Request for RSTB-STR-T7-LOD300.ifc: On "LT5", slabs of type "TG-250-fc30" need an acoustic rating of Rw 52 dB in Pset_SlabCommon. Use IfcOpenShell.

First a look at what the model holds.

```python
import ifcopenshell
import ifcopenshell.util.element

model = ifcopenshell.open("RSTB-STR-T7-LOD300.ifc")
print(model.schema)
storey = next(s for s in model.by_type("IfcBuildingStorey") if s.Name == "LT5")
slabs = [e for e in ifcopenshell.util.element.get_decomposition(storey) if e.is_a("IfcSlab")]
seen = {}
for e in slabs:
    element_type = ifcopenshell.util.element.get_type(e)
    key = (element_type.Name if element_type != e and element_type else None, ifcopenshell.util.element.get_pset(e, "Pset_SlabCommon", "AcousticRating"))
    seen[key] = seen.get(key, 0) + 1
for (name, value), count in sorted(seen.items(), key=str):
    print(count, "x", name, "|", value)
```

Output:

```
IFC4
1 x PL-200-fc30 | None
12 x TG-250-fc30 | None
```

```python
import ifcopenshell
import ifcopenshell.api.pset
import ifcopenshell.util.element

model = ifcopenshell.open("RSTB-STR-T7-LOD300.ifc")

storey = next(s for s in model.by_type("IfcBuildingStorey") if s.Name == "LT5")
slabs = [e for e in ifcopenshell.util.element.get_decomposition(storey) if e.is_a("IfcSlab")]

count = 0
for e in slabs:
    element_type = ifcopenshell.util.element.get_type(e)
    if element_type in (None, e) or element_type.Name != "TG-250-fc30":
        continue
    # add_pset returns the element's existing set when there is one.
    pset = ifcopenshell.api.pset.add_pset(model, product=e, name="Pset_SlabCommon")
    ifcopenshell.api.pset.edit_pset(model, pset=pset, properties={"AcousticRating": "Rw 52 dB"})
    count += 1

print(count, "slabs updated")

model.write("RSTB-STR-T7-LOD300_edited.ifc")
```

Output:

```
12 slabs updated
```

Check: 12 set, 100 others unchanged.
